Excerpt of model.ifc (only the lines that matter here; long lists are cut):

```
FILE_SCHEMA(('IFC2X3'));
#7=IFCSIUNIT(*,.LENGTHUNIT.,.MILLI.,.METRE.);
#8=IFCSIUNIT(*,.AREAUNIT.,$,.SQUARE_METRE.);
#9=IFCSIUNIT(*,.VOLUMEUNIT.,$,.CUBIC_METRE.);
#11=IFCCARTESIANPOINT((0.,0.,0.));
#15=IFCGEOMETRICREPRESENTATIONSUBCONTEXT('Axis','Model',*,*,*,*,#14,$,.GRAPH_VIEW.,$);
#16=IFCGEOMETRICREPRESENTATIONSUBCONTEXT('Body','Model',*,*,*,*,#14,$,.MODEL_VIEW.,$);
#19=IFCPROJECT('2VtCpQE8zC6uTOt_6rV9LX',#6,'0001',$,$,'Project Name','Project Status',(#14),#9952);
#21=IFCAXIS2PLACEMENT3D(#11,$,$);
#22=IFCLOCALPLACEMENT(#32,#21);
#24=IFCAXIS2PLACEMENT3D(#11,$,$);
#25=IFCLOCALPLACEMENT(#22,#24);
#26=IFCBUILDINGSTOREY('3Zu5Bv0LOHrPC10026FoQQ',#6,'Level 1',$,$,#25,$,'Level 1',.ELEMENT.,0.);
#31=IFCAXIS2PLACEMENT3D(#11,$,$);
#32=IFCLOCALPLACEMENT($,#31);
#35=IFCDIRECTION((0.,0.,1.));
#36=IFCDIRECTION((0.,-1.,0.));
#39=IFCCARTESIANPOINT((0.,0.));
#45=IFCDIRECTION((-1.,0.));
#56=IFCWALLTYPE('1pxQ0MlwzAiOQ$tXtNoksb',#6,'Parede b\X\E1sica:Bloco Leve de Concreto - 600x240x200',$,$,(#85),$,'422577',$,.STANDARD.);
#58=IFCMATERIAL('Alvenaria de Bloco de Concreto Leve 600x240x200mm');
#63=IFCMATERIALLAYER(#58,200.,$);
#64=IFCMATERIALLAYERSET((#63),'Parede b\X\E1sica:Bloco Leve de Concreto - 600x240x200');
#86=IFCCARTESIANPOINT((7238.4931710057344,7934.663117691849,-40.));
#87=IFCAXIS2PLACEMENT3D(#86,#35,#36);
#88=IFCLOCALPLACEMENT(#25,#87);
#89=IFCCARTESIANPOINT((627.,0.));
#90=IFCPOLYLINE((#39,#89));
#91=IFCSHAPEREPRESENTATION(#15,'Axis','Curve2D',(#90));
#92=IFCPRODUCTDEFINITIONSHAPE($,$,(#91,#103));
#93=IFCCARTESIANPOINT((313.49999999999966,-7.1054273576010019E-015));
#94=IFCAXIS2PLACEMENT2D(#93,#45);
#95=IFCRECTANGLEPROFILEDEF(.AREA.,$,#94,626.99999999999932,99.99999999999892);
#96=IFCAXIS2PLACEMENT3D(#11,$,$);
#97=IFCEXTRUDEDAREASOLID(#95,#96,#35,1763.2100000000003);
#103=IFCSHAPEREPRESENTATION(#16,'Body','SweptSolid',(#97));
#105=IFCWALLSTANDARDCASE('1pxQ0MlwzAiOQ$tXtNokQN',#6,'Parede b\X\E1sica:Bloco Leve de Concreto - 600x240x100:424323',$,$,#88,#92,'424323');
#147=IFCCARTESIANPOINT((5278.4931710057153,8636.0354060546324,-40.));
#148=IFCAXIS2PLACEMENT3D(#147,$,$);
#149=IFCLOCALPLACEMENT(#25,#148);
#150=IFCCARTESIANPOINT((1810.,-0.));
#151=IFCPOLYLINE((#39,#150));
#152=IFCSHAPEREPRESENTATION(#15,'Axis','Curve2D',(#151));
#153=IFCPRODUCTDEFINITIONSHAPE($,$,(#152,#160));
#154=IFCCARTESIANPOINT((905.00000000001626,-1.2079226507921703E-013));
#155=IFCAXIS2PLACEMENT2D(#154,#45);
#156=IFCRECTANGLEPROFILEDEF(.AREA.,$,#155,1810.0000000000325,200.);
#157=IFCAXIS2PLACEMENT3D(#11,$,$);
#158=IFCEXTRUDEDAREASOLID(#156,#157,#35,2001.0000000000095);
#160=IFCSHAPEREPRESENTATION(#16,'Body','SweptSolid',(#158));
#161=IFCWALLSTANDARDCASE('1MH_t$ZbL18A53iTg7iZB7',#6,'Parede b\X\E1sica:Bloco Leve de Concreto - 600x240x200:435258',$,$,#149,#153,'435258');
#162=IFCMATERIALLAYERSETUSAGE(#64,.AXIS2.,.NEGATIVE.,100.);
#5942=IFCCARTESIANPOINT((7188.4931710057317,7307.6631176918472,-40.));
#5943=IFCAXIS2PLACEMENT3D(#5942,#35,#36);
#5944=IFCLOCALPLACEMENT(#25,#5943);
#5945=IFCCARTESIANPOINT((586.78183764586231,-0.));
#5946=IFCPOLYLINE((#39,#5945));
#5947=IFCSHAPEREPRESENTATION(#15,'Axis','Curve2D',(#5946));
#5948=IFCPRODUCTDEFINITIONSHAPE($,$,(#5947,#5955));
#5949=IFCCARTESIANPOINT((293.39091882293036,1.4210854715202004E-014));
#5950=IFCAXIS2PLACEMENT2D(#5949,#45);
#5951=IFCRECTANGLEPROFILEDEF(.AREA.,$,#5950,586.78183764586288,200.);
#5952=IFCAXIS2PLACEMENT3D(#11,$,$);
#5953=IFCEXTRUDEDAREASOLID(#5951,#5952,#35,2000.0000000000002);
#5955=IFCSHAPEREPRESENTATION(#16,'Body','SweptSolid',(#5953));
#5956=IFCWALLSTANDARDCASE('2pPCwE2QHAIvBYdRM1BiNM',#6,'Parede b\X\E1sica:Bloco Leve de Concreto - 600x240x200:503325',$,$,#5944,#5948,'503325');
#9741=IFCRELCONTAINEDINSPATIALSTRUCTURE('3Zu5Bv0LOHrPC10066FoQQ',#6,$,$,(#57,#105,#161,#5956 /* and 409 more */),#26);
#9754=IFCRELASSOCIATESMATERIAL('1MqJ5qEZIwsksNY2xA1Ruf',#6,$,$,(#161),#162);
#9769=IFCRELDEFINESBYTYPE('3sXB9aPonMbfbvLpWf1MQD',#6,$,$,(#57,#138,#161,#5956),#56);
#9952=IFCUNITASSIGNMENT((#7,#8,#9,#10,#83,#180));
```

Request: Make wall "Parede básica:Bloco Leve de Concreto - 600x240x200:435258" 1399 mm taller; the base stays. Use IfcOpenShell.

```python
import ifcopenshell
import ifcopenshell.geom
import ifcopenshell.util.representation
import ifcopenshell.util.shape
import ifcopenshell.util.unit

model = ifcopenshell.open("model.ifc")
unit_scale = ifcopenshell.util.unit.calculate_unit_scale(model)
settings = ifcopenshell.geom.settings()


def volume(element):
    """Net volume in cubic metres, openings subtracted."""
    shape = ifcopenshell.geom.create_shape(settings, element)
    return ifcopenshell.util.shape.get_volume(shape.geometry)


wall = model.by_guid("1MH_t$ZbL18A53iTg7iZB7")
before = volume(wall)

body = ifcopenshell.util.representation.get_representation(wall, "Model", "Body")
solid = body.Items[0]
old_height = solid.Depth
solid.Depth += 1.399 / unit_scale
after = volume(wall)

print(f"height {old_height:g} -> {solid.Depth:g}, volume {before:.3f} -> {after:.3f} m3")

model.write("model_updated.ifc")
```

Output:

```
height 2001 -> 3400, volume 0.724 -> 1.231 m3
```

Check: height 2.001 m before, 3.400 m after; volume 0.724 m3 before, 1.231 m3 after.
